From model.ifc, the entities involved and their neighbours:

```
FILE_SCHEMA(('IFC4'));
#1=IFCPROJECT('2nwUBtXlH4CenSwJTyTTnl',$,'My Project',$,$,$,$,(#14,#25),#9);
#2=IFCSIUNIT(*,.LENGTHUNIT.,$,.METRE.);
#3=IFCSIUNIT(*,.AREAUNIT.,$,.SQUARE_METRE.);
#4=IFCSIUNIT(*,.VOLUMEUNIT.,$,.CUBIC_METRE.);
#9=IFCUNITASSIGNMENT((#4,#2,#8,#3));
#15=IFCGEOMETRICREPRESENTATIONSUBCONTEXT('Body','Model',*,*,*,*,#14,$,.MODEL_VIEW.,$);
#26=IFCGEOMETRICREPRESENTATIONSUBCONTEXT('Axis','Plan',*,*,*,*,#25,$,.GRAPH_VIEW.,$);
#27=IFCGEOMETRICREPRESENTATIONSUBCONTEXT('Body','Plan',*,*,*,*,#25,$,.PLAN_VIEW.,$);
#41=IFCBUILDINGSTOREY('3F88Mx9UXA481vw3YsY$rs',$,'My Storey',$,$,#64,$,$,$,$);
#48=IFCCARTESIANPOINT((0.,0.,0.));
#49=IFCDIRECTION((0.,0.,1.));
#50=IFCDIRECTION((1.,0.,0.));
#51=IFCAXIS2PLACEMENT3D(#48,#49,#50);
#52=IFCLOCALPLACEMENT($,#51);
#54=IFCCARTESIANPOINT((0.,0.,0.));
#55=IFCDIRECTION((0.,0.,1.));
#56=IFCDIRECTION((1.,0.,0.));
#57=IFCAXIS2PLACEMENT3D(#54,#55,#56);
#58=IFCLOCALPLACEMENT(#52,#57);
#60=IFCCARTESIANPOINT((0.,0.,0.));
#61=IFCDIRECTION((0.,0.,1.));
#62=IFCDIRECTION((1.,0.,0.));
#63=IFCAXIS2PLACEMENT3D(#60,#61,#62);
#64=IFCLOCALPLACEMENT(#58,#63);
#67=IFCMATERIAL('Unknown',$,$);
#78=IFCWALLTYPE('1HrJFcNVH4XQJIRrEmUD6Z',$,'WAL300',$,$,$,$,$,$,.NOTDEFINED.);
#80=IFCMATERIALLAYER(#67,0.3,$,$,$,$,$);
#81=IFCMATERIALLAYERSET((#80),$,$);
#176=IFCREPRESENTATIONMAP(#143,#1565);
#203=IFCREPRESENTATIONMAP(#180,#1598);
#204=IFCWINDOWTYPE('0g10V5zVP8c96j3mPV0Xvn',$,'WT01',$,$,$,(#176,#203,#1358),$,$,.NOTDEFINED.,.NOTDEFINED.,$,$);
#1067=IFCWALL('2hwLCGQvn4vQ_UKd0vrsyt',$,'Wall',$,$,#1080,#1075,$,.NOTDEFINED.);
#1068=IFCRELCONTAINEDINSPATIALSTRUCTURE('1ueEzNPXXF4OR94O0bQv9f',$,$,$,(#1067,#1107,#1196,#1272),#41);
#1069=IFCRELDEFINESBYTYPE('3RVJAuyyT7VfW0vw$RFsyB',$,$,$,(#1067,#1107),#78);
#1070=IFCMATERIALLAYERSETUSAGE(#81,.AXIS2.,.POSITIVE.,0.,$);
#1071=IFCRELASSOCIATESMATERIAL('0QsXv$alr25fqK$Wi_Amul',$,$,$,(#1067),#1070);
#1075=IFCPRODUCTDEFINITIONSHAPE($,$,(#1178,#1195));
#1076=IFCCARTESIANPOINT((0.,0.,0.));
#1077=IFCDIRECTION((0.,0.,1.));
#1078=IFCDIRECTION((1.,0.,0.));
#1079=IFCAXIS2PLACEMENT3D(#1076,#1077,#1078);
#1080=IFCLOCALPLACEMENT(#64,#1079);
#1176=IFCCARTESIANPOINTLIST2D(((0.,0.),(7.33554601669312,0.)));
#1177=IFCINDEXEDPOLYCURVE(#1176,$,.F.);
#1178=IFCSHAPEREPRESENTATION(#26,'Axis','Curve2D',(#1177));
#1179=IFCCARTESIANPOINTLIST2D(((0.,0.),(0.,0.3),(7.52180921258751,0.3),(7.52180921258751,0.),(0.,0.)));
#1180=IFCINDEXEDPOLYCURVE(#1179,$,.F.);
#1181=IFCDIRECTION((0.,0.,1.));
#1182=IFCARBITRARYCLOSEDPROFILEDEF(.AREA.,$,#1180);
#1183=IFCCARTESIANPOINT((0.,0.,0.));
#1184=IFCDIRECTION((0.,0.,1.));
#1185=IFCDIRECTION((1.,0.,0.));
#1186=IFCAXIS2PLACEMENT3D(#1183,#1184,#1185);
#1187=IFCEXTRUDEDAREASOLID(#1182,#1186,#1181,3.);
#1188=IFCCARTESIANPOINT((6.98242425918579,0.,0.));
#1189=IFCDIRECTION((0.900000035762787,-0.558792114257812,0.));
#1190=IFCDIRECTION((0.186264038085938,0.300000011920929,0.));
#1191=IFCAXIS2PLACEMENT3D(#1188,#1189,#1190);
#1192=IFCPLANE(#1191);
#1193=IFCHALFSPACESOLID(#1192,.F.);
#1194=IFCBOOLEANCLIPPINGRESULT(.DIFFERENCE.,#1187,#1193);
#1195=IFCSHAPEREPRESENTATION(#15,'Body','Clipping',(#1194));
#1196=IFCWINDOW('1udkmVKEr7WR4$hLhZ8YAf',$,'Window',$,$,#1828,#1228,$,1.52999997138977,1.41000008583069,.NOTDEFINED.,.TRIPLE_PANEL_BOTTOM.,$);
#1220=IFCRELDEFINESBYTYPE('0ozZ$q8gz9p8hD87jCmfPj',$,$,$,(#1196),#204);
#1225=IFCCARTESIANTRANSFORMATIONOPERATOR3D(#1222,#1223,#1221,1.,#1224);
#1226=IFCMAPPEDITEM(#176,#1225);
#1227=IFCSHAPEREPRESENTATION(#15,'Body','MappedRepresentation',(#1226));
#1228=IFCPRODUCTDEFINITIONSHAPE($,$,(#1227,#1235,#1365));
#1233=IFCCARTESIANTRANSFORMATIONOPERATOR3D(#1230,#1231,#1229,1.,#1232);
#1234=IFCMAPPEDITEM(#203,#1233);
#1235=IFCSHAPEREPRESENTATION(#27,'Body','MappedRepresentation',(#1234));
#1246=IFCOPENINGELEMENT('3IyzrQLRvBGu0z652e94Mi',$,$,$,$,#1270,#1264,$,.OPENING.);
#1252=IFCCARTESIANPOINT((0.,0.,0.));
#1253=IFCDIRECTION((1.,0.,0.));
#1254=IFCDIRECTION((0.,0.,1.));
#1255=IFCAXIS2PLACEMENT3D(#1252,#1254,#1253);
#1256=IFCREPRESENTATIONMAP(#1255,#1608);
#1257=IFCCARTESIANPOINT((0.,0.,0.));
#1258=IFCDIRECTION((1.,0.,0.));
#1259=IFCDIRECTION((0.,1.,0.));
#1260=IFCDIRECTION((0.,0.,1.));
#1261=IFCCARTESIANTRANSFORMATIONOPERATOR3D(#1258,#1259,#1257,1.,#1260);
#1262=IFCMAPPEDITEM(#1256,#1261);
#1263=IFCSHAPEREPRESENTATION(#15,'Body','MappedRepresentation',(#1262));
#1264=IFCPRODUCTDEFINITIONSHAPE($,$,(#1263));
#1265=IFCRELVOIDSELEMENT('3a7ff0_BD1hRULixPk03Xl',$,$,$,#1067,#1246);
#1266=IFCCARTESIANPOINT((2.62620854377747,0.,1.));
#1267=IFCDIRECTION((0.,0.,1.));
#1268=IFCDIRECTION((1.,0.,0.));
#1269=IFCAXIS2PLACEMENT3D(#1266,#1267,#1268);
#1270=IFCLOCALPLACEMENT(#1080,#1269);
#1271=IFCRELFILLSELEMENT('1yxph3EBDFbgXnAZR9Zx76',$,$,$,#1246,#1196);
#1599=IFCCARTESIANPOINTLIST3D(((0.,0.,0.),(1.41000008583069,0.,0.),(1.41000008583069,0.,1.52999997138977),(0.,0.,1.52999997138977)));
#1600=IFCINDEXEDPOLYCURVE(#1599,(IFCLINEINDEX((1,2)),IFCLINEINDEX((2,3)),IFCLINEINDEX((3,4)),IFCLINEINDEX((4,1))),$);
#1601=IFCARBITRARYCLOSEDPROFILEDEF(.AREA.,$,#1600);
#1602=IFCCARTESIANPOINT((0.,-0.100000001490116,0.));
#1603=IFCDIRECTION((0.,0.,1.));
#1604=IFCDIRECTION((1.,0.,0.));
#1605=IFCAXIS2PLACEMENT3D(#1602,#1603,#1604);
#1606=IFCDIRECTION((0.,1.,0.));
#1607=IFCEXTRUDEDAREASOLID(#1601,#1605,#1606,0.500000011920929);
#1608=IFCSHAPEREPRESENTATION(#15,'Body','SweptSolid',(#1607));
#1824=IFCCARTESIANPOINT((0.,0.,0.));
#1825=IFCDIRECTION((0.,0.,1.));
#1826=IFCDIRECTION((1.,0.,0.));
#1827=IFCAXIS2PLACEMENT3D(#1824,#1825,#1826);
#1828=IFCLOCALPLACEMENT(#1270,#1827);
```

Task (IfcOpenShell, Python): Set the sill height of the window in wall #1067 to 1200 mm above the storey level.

```python
import numpy as np
import ifcopenshell
import ifcopenshell.api.geometry
import ifcopenshell.geom
import ifcopenshell.util.element
import ifcopenshell.util.placement
import ifcopenshell.util.shape
import ifcopenshell.util.unit

model = ifcopenshell.open("model.ifc")
unit_scale = ifcopenshell.util.unit.calculate_unit_scale(model)

window = model.by_guid("1udkmVKEr7WR4$hLhZ8YAf")
opening = window.FillsVoids[0].RelatingOpeningElement
storey = ifcopenshell.util.element.get_container(window, ifc_class="IfcBuildingStorey")
level = ifcopenshell.util.placement.get_local_placement(storey.ObjectPlacement)[2, 3]

# The opening's origin need not be at the sill, so measure its lowest point.
shape = ifcopenshell.geom.create_shape(ifcopenshell.geom.settings(), opening)
bottom = ifcopenshell.util.shape.get_shape_bottom_elevation(shape, shape.geometry) / unit_scale
dz = level + 1.2 / unit_scale - bottom

shift = np.array([0.0, 0.0, dz])
# The window is placed relative to its opening, so it follows when the opening moves.
matrix = ifcopenshell.util.placement.get_local_placement(opening.ObjectPlacement)
matrix[:3, 3] += shift
ifcopenshell.api.geometry.edit_object_placement(
    model, product=opening, matrix=matrix, is_si=False, should_transform_children=True
)

print(f"moved by {dz * unit_scale:+.3f} m")

model.write("model_rev.ifc")
```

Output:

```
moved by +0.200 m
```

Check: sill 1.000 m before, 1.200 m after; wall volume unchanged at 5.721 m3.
